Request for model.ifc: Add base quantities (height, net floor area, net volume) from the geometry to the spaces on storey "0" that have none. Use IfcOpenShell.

First a look at what the model holds.

```python
import ifcopenshell
import ifcopenshell.util.element
import ifcopenshell.util.unit

model = ifcopenshell.open("model.ifc")
print(model.schema)
for unit_type in ("LENGTHUNIT", "AREAUNIT", "VOLUMEUNIT"):
    print(unit_type, ifcopenshell.util.unit.calculate_unit_scale(model, unit_type))
storey = next(s for s in model.by_type("IfcBuildingStorey") if s.Name == "0")
spaces = [e for e in ifcopenshell.util.element.get_decomposition(storey) if e.is_a("IfcSpace")]
for e in sorted(spaces, key=lambda e: e.id()):
    print(e.id(), e.is_a(), e.Name, list(ifcopenshell.util.element.get_psets(e, qtos_only=True)), sep=" | ")
```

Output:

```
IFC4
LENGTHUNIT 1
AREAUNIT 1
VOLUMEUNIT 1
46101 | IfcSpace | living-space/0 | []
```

```python
import ifcopenshell
import ifcopenshell.api.pset
import ifcopenshell.geom
import ifcopenshell.util.element
import ifcopenshell.util.shape
import ifcopenshell.util.unit

model = ifcopenshell.open("model.ifc")
unit_scale = ifcopenshell.util.unit.calculate_unit_scale(model)
area_scale = ifcopenshell.util.unit.calculate_unit_scale(model, "AREAUNIT")
volume_scale = ifcopenshell.util.unit.calculate_unit_scale(model, "VOLUMEUNIT")
settings = ifcopenshell.geom.settings()

storey = next(s for s in model.by_type("IfcBuildingStorey") if s.Name == "0")
spaces = [e for e in ifcopenshell.util.element.get_decomposition(storey) if e.is_a("IfcSpace")]

for e in sorted(spaces, key=lambda e: e.id()):
    if ifcopenshell.util.element.get_psets(e, qtos_only=True, should_inherit=False):
        continue
    # Geometry comes back in metres, in the element's own axes.
    shape = ifcopenshell.geom.create_shape(settings, e)
    values = {
        "Height": ifcopenshell.util.shape.get_z(shape.geometry) / unit_scale,
        "NetFloorArea": ifcopenshell.util.shape.get_footprint_area(shape.geometry) / area_scale,
        "NetVolume": ifcopenshell.util.shape.get_volume(shape.geometry) / volume_scale,
    }
    qto = ifcopenshell.api.pset.add_qto(model, product=e, name="Qto_SpaceBaseQuantities")
    ifcopenshell.api.pset.edit_qto(model, qto=qto, properties=values)
    print(e.id(), {k: round(v, 3) for k, v in values.items()})

model.write("model_edited.ifc")
```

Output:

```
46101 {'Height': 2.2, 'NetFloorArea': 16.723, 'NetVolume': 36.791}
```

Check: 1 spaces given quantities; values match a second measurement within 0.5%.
